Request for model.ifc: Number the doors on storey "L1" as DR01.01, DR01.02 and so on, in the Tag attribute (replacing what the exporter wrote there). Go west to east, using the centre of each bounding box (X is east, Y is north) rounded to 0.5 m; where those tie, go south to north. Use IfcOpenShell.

First a look at what the model holds.

```python
import ifcopenshell
import ifcopenshell.util.element
import ifcopenshell.util.placement

model = ifcopenshell.open("model.ifc")
print(model.schema)
storey = next(s for s in model.by_type("IfcBuildingStorey") if s.Name == "L1")
doors = [e for e in ifcopenshell.util.element.get_decomposition(storey) if e.is_a("IfcDoor")]
for e in sorted(doors, key=lambda e: e.id()):
    origin = ifcopenshell.util.placement.get_local_placement(e.ObjectPlacement)[:3, 3]
    print(e.id(), e.Tag, e.Name, origin.round(2) + 0.0, sep=" | ")
```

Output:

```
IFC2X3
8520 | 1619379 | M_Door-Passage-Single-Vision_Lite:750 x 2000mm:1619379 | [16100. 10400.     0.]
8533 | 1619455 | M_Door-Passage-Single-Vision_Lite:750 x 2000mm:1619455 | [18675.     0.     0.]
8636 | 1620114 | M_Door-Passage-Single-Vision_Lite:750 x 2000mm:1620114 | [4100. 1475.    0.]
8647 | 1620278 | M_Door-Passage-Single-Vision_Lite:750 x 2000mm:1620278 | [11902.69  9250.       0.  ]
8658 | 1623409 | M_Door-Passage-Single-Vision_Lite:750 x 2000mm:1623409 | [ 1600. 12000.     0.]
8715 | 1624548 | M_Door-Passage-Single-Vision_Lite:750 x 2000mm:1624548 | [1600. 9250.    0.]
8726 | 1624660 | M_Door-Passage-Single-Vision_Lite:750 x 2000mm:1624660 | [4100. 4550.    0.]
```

```python
import ifcopenshell
import ifcopenshell.geom
import ifcopenshell.util.element
import ifcopenshell.util.shape

model = ifcopenshell.open("model.ifc")
settings = ifcopenshell.geom.settings()
settings.set("use-world-coords", True)


def centre(element):
    shape = ifcopenshell.geom.create_shape(settings, element)
    return ifcopenshell.util.shape.get_bbox_centroid(shape.geometry)


storey = next(s for s in model.by_type("IfcBuildingStorey") if s.Name == "L1")
doors = [e for e in ifcopenshell.util.element.get_decomposition(storey) if e.is_a("IfcDoor")]

# Insertion points can sit at a corner or the storey origin, so sort by the geometry (in metres).
centres = {e: centre(e) for e in doors}
doors.sort(key=lambda e: (round(centres[e][0] / 0.5), centres[e][1]))

for i, e in enumerate(doors, start=1):
    number = f"DR01.{i:02d}"
    e.Tag = number
    print(e.id(), number)

model.write("model-out.ifc")
```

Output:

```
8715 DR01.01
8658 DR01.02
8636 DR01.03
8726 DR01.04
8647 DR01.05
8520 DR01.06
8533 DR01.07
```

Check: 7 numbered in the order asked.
